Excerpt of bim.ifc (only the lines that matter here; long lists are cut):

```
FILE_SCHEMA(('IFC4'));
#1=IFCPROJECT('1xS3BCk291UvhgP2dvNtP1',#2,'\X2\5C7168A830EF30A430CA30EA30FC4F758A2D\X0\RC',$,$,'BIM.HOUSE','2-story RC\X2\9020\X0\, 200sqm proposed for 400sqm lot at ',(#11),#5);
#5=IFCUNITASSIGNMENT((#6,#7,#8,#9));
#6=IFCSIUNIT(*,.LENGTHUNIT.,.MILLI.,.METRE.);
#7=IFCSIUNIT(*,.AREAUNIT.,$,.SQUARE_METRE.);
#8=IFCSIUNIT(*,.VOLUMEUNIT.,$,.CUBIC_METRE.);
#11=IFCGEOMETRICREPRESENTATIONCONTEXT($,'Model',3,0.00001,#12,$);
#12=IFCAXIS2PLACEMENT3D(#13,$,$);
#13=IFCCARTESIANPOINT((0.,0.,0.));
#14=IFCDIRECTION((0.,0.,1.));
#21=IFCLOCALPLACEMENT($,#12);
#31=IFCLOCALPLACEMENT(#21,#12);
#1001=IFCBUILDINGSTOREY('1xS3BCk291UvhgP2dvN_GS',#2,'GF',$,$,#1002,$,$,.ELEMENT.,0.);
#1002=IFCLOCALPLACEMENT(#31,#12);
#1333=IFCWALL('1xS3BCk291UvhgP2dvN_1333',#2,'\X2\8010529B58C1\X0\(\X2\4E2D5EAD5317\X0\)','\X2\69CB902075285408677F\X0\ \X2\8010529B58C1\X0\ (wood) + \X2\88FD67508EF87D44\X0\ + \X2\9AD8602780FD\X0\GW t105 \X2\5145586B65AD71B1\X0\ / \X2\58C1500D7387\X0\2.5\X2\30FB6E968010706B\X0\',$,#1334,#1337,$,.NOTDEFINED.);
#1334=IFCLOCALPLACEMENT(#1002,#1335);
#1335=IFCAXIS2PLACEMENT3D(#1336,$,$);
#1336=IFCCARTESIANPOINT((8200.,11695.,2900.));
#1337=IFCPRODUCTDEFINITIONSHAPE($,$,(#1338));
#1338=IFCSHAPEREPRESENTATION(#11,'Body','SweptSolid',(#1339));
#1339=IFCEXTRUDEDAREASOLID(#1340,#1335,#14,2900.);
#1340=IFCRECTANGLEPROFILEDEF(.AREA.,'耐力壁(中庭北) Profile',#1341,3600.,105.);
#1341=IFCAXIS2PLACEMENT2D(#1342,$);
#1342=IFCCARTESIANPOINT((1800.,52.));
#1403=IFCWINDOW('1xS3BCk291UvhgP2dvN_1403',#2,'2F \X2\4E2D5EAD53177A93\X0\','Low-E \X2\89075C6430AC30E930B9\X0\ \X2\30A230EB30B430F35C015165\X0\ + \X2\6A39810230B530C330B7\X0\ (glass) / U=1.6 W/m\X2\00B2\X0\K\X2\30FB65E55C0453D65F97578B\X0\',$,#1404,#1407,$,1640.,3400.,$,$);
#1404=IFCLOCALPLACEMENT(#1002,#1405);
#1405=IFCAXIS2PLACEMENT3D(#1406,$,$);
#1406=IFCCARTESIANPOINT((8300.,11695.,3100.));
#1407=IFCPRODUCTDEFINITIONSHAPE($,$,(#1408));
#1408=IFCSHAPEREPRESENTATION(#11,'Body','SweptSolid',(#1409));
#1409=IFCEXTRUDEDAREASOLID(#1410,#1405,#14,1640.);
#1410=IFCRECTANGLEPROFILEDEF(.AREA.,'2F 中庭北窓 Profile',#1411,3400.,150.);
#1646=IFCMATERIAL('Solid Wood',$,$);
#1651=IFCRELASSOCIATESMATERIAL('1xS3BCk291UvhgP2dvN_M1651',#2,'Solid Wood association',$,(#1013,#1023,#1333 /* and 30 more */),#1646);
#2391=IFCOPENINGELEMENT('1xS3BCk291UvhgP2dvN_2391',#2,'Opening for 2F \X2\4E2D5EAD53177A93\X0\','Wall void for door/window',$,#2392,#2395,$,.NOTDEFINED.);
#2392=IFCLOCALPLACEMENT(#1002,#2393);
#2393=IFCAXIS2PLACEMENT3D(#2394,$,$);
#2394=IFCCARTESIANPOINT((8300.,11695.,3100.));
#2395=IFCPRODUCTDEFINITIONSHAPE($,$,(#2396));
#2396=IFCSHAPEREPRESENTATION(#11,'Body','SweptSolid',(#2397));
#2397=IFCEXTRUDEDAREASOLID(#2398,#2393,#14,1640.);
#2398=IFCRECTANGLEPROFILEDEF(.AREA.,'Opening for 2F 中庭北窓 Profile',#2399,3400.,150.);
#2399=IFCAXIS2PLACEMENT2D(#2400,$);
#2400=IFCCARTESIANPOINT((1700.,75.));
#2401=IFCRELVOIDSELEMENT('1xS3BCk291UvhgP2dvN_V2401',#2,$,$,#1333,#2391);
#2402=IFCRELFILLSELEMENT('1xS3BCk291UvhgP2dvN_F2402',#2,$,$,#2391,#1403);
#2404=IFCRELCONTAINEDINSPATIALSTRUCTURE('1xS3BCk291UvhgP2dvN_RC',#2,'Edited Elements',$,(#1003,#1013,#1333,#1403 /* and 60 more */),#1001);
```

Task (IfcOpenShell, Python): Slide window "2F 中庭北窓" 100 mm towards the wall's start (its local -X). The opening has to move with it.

```python
import ifcopenshell
import ifcopenshell.api.geometry
import ifcopenshell.util.placement
import ifcopenshell.util.unit

model = ifcopenshell.open("bim.ifc")
unit_scale = ifcopenshell.util.unit.calculate_unit_scale(model)

window = model.by_guid("1xS3BCk291UvhgP2dvN_1403")
opening = window.FillsVoids[0].RelatingOpeningElement
wall = opening.VoidsElements[0].RelatingBuildingElement

wall_matrix = ifcopenshell.util.placement.get_local_placement(wall.ObjectPlacement)
shift = wall_matrix[:3, 0] * -0.1 / unit_scale
before = ifcopenshell.util.placement.get_local_placement(window.ObjectPlacement)[:3, 3].copy()

# The window is not placed relative to its opening, so move both.
for product in (opening, window):
    matrix = ifcopenshell.util.placement.get_local_placement(product.ObjectPlacement)
    matrix[:3, 3] += shift
    ifcopenshell.api.geometry.edit_object_placement(model, product=product, matrix=matrix, is_si=False)

after = ifcopenshell.util.placement.get_local_placement(window.ObjectPlacement)[:3, 3]
print("window moved by", (after - before).round(3) + 0.0)

model.write("bim_updated.ifc")
```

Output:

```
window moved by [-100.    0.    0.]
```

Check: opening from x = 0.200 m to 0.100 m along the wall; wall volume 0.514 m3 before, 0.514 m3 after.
